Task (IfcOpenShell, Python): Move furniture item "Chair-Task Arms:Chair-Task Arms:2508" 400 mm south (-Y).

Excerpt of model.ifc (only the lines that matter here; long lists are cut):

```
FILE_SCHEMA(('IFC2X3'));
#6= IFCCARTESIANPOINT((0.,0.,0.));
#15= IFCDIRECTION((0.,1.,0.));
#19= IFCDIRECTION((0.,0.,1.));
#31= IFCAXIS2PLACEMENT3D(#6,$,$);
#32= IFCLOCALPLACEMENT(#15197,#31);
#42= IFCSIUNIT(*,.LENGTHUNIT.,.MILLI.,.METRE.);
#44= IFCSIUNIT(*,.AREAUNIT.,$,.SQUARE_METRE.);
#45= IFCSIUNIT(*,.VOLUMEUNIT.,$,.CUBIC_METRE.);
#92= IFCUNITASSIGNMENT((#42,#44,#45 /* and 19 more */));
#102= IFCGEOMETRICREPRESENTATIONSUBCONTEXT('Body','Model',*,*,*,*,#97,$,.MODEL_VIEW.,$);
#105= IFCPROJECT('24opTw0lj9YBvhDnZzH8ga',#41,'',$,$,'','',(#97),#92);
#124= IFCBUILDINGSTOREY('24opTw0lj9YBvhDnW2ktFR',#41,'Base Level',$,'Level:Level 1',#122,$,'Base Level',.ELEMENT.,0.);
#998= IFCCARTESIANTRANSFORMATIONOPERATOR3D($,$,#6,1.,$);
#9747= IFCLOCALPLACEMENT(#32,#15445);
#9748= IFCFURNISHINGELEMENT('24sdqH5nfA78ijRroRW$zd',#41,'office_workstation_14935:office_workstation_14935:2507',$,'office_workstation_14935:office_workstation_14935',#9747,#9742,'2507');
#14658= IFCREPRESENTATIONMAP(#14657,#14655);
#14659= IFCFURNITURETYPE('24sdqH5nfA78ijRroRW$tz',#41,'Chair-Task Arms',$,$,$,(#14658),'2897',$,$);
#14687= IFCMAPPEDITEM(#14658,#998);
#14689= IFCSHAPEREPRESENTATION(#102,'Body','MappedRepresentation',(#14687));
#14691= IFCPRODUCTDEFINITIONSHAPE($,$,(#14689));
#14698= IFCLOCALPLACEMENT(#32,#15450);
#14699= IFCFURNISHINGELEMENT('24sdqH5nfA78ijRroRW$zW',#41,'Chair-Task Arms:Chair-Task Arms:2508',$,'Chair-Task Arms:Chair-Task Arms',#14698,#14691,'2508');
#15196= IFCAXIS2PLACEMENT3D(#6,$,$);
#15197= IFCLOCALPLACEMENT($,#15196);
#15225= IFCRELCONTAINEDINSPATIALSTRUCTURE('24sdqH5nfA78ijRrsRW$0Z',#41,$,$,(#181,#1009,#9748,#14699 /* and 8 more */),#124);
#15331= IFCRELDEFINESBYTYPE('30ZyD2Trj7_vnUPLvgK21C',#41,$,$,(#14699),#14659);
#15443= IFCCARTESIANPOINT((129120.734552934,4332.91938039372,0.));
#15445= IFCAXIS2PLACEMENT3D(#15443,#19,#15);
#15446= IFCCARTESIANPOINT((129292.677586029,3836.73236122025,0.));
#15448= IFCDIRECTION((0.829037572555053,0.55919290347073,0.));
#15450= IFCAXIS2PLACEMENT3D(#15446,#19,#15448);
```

```python
import ifcopenshell
import ifcopenshell.api.geometry
import ifcopenshell.util.placement

model = ifcopenshell.open("model.ifc")

item = model.by_guid("24sdqH5nfA78ijRroRW$zW")
matrix = ifcopenshell.util.placement.get_local_placement(item.ObjectPlacement)
matrix[1, 3] -= 400.0
ifcopenshell.api.geometry.edit_object_placement(model, product=item, matrix=matrix, is_si=False)

print(ifcopenshell.util.placement.get_local_placement(item.ObjectPlacement).round(3) + 0.0)

model.write("model_rev.ifc")
```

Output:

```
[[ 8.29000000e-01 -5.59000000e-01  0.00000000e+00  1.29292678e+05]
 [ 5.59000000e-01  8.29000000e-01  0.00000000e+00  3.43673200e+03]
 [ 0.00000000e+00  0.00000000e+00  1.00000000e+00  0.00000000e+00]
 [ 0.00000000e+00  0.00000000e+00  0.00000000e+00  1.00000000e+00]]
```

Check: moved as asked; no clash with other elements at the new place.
